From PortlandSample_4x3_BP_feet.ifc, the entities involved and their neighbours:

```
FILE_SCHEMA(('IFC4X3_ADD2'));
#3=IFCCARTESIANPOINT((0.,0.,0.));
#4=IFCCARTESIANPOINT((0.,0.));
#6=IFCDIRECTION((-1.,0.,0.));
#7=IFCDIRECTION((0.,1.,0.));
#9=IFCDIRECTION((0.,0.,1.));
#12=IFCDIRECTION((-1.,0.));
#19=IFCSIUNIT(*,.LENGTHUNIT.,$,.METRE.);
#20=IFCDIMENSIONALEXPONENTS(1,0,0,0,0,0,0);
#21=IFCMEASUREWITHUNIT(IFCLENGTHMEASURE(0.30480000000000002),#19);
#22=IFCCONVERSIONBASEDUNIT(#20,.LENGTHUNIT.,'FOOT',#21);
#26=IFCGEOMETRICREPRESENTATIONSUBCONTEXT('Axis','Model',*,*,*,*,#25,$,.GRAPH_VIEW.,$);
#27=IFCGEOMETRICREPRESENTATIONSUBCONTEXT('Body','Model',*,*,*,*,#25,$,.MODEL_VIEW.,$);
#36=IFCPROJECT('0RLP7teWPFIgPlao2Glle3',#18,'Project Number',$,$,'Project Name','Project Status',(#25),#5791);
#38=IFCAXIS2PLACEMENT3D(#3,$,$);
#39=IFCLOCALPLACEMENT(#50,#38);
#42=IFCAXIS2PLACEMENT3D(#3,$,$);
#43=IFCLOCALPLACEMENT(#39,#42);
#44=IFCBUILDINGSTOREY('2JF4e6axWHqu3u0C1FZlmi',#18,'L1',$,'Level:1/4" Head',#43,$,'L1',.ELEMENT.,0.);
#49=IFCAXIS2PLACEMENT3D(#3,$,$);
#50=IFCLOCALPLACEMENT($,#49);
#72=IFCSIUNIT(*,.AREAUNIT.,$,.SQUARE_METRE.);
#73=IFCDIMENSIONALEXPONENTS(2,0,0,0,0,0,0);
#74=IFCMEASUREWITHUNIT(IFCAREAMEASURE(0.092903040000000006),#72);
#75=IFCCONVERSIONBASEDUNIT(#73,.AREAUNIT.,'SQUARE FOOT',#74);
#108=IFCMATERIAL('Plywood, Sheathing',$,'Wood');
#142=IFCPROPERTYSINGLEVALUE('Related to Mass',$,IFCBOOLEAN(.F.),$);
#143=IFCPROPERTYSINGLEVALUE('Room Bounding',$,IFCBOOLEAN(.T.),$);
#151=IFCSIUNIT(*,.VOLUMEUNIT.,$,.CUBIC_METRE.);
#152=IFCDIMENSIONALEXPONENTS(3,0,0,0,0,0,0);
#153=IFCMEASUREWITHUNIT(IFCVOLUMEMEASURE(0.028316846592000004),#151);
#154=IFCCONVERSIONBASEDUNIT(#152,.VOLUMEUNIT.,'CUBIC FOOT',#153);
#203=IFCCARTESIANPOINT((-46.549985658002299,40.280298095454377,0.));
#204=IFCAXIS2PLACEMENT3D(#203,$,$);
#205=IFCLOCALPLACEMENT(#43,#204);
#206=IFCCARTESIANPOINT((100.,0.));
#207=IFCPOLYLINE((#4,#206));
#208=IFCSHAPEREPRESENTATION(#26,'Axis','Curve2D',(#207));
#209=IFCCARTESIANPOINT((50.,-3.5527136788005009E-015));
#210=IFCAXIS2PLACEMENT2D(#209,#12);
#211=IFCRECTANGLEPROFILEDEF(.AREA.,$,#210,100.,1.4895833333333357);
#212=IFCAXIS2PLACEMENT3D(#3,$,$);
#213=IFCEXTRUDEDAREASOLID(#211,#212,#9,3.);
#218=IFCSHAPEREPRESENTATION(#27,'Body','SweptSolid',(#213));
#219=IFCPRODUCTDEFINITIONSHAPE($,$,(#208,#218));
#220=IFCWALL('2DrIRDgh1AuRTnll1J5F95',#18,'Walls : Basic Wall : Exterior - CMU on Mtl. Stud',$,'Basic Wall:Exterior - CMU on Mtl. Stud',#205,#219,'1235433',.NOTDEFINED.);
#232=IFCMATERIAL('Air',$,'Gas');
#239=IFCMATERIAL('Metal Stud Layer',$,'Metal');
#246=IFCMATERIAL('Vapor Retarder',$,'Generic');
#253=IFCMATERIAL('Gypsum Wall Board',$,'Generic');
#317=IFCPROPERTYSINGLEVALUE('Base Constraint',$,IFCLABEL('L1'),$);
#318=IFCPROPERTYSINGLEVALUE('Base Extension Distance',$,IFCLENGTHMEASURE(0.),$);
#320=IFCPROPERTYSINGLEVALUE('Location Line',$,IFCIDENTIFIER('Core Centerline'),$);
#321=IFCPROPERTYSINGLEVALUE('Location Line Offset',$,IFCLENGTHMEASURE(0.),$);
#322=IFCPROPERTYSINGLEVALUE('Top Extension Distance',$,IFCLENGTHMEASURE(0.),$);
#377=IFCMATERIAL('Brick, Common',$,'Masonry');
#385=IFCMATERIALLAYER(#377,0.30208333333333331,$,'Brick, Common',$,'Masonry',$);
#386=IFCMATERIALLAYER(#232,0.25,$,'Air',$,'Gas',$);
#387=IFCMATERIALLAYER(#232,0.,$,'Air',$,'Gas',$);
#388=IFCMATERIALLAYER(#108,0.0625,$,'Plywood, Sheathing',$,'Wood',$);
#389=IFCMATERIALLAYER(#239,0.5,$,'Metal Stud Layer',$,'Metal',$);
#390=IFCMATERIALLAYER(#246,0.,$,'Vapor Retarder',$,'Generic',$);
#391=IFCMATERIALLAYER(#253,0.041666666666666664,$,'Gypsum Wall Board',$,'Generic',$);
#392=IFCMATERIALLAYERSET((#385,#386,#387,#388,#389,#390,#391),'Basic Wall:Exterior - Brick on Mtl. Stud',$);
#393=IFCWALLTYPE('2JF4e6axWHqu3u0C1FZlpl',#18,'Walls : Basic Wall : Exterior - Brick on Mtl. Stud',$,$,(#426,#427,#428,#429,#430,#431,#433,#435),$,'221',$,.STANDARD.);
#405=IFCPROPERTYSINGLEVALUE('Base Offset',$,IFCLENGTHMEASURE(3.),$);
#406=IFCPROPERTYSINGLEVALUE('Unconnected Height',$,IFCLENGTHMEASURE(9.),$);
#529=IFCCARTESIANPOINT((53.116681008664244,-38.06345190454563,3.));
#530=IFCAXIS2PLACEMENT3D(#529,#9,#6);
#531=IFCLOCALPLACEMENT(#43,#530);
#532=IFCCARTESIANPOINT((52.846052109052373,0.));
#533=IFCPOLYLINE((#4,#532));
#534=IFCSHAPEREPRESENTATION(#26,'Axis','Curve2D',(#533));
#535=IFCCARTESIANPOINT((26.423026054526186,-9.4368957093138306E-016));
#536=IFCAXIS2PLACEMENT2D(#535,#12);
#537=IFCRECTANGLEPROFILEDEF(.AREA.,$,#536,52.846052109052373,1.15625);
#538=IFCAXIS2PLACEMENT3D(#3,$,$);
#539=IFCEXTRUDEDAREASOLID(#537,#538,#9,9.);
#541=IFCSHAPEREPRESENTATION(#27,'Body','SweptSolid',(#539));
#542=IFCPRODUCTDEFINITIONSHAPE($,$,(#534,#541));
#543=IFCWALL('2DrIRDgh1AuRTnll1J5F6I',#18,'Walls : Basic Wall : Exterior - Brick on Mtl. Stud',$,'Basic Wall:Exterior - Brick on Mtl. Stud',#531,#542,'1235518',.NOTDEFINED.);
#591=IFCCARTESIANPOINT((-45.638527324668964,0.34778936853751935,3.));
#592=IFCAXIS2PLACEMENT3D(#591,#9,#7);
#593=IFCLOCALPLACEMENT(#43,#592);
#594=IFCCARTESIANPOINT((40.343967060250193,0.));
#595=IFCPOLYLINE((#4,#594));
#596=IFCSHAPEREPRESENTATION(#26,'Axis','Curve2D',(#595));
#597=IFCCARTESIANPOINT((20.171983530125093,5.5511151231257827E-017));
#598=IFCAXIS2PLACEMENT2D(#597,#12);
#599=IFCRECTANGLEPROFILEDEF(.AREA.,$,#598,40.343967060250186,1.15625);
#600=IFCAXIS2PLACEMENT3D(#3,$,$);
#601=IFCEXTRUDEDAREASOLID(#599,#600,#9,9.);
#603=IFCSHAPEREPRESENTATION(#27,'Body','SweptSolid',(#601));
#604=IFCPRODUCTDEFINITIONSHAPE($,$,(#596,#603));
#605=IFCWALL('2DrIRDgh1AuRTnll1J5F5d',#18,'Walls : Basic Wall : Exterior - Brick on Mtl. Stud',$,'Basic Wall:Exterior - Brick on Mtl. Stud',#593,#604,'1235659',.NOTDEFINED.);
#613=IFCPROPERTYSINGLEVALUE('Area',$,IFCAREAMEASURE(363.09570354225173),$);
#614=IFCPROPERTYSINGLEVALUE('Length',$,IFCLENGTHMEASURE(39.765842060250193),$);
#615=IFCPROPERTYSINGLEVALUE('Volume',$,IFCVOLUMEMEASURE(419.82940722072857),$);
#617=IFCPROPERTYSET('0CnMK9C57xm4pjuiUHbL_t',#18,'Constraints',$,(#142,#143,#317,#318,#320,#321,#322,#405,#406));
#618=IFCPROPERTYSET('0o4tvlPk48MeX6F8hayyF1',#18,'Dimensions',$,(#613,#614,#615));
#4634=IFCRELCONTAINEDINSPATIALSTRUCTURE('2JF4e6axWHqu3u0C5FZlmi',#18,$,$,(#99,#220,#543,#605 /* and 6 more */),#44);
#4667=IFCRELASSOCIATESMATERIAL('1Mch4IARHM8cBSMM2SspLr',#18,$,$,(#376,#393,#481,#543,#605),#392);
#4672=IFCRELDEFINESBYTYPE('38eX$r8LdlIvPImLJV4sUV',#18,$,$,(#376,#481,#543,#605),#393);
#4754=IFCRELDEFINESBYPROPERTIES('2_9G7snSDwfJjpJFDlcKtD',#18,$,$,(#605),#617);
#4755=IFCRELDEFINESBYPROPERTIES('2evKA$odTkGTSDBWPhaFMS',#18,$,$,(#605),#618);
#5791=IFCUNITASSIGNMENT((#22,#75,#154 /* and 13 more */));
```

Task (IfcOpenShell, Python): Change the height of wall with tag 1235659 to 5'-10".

```python
import ifcopenshell
import ifcopenshell.api.pset
import ifcopenshell.geom
import ifcopenshell.util.element
import ifcopenshell.util.representation
import ifcopenshell.util.shape
import ifcopenshell.util.unit

model = ifcopenshell.open("PortlandSample_4x3_BP_feet.ifc")
unit_scale = ifcopenshell.util.unit.calculate_unit_scale(model)
area_scale = ifcopenshell.util.unit.calculate_unit_scale(model, "AREAUNIT")
volume_scale = ifcopenshell.util.unit.calculate_unit_scale(model, "VOLUMEUNIT")
settings = ifcopenshell.geom.settings()


def volume(element):
    """Net volume in cubic metres, openings subtracted."""
    shape = ifcopenshell.geom.create_shape(settings, element)
    return ifcopenshell.util.shape.get_volume(shape.geometry)


wall = model.by_guid("2DrIRDgh1AuRTnll1J5F5d")
before = volume(wall)

body = ifcopenshell.util.representation.get_representation(wall, "Model", "Body")
solid = body.Items[0]
old_height = solid.Depth
solid.Depth = 70 * 0.0254 / unit_scale
after = volume(wall)
thickness = 0.3524  # wall thickness in metres

# Update the stored height, areas and volumes.
pset = model.by_id(ifcopenshell.util.element.get_pset(wall, "Constraints", should_inherit=False)["id"])
ifcopenshell.api.pset.edit_pset(model, pset=pset, properties={
    "Unconnected Height": model.create_entity("IfcLengthMeasure", solid.Depth),
})
pset = model.by_id(ifcopenshell.util.element.get_pset(wall, "Dimensions", should_inherit=False)["id"])
ifcopenshell.api.pset.edit_pset(model, pset=pset, properties={
    "Area": model.create_entity("IfcAreaMeasure", after / thickness / area_scale),
    "Volume": model.create_entity("IfcVolumeMeasure", after / volume_scale),
})

print(f"height {old_height:g} -> {solid.Depth:g}, volume {before:.3f} -> {after:.3f} m3")

model.write("PortlandSample_4x3_BP_feet-out.ifc")
```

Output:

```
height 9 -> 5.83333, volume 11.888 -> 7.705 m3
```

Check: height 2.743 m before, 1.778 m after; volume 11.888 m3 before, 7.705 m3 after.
